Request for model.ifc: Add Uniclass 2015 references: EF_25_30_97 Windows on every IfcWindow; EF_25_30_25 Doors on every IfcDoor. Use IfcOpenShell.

First a look at what the model holds.

```python
import ifcopenshell

model = ifcopenshell.open("model.ifc")
print(model.schema)
print("classifications:", [c.Name for c in model.by_type("IfcClassification")])
for ifc_class in ("IfcDoor", "IfcRoof", "IfcStair", "IfcWall", "IfcWindow"):
    print(ifc_class, len(model.by_type(ifc_class)))
```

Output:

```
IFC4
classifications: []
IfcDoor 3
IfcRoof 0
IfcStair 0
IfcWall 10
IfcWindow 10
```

```python
import ifcopenshell
import ifcopenshell.api.classification

model = ifcopenshell.open("model.ifc")

system = ifcopenshell.api.classification.add_classification(model, classification="Uniclass 2015")

codes = {
    "IfcWindow": ("EF_25_30_97", "Windows"),
    "IfcDoor": ("EF_25_30_25", "Doors"),
}
for ifc_class, (code, name) in codes.items():
    products = model.by_type(ifc_class)
    ifcopenshell.api.classification.add_reference(
        model, products=products, classification=system, identification=code, name=name
    )
    print(code, len(products))

model.write("model-out.ifc")
```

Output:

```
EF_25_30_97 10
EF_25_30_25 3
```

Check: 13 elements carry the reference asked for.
